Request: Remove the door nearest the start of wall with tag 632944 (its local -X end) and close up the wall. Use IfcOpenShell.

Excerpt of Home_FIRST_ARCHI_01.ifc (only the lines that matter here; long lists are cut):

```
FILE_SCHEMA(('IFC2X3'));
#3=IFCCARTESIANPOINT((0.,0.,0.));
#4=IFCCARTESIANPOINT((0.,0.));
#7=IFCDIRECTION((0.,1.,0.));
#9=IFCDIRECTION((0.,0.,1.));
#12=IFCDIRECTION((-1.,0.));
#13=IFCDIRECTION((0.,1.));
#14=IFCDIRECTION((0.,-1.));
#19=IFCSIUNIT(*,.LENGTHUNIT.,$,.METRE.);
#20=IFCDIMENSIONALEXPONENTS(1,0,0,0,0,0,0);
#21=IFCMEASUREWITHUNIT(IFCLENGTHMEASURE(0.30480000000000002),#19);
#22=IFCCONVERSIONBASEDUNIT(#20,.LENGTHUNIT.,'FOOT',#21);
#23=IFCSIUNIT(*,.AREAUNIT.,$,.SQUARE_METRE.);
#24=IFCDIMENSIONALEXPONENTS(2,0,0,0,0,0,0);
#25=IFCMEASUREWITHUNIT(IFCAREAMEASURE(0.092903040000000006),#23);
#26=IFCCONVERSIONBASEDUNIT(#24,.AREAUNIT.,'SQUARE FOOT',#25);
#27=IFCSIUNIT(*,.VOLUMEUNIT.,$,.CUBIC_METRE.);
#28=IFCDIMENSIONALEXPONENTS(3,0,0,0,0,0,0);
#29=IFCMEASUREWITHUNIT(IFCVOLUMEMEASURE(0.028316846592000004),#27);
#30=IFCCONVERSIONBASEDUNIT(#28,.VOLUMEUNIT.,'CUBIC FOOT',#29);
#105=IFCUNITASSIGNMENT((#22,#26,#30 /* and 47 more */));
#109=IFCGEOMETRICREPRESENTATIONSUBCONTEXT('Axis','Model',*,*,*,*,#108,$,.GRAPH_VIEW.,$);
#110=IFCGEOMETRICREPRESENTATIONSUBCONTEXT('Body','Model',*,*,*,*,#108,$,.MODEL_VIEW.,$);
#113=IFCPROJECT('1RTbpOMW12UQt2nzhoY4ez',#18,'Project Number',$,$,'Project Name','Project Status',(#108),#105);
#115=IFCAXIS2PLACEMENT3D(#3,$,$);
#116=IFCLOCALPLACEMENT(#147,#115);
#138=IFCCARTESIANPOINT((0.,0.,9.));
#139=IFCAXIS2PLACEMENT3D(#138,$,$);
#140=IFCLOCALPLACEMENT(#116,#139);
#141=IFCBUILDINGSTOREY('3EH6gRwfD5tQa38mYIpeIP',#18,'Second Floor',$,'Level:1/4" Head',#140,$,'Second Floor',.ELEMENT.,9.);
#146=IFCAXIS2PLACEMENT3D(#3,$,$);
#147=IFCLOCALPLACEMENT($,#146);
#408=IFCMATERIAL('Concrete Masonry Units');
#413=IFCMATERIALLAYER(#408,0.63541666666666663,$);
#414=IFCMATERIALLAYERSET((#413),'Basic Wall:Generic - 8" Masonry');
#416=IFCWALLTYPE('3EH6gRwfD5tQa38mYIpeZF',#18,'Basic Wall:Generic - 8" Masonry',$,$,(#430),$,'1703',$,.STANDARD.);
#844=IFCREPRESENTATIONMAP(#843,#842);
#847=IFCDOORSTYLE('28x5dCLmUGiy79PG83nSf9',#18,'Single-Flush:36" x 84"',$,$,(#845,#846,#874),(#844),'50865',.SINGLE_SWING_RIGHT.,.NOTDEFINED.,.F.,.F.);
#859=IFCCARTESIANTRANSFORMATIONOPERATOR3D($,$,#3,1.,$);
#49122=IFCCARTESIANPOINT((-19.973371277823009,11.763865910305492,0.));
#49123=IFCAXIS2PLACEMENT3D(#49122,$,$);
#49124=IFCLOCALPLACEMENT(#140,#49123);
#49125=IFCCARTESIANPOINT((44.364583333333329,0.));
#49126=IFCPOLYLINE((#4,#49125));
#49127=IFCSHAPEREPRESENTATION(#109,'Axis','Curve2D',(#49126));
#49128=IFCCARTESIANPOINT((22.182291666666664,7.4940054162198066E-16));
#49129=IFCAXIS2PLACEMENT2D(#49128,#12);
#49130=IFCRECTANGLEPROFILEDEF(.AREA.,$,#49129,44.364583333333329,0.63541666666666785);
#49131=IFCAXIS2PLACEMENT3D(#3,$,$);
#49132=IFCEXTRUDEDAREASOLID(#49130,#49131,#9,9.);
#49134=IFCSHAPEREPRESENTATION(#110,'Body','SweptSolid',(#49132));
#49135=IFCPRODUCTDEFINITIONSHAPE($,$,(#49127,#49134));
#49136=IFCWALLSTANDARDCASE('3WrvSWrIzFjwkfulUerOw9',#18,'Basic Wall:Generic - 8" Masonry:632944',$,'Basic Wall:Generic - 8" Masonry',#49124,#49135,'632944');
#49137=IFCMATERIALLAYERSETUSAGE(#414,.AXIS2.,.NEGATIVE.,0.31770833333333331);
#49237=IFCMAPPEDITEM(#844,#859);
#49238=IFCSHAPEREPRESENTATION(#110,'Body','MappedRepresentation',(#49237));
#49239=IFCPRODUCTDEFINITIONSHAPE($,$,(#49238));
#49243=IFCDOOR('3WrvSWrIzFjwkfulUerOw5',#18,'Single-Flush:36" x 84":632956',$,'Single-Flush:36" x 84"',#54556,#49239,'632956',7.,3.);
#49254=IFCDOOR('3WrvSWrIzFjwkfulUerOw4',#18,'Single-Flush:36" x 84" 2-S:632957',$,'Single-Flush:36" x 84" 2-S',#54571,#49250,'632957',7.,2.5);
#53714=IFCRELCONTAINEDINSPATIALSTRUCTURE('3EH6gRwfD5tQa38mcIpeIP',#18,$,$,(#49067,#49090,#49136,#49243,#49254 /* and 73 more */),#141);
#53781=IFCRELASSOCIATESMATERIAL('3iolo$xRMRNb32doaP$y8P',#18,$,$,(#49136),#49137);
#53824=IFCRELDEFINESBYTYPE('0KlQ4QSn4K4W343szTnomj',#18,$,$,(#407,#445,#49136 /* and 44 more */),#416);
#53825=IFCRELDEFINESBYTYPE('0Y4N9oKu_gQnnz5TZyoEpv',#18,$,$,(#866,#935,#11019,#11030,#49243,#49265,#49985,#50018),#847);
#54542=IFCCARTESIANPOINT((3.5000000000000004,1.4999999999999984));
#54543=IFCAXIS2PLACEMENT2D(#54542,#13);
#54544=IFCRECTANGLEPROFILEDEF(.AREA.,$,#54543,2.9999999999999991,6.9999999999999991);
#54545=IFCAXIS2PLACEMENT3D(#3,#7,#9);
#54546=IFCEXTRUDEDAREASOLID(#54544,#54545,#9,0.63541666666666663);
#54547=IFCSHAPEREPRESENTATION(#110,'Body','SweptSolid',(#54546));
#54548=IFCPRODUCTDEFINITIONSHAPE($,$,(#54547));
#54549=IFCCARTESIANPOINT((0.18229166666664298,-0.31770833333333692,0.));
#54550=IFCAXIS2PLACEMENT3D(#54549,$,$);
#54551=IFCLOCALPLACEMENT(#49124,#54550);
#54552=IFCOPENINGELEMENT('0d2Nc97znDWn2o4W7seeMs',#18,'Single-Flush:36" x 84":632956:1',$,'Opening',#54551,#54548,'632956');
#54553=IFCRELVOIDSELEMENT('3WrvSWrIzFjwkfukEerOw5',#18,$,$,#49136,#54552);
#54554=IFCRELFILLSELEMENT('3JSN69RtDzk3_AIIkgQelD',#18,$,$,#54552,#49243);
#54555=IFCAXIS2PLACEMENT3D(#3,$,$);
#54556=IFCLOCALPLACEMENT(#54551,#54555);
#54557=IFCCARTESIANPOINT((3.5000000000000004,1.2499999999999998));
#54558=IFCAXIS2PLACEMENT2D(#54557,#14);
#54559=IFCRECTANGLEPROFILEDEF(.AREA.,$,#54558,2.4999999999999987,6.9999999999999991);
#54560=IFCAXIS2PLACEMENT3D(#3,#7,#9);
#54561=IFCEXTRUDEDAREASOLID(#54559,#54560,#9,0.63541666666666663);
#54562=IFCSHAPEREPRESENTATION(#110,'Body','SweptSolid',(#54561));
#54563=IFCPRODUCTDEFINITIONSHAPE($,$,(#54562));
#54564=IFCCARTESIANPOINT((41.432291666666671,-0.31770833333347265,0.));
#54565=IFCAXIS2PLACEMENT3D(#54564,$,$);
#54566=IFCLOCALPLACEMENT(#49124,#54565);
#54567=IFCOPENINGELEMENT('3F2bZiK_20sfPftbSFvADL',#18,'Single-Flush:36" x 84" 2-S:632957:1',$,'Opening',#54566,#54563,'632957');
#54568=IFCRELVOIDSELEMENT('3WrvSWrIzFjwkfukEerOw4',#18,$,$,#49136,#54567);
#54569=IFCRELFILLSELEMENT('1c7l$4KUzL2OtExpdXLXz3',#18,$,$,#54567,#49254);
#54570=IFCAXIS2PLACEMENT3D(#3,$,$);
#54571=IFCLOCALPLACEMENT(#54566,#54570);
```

```python
import ifcopenshell
import ifcopenshell.api.feature
import ifcopenshell.api.root
import ifcopenshell.geom
import ifcopenshell.util.shape

model = ifcopenshell.open("Home_FIRST_ARCHI_01.ifc")
settings = ifcopenshell.geom.settings()


def volume(element):
    """Net volume in cubic metres, openings subtracted."""
    shape = ifcopenshell.geom.create_shape(settings, element)
    return ifcopenshell.util.shape.get_volume(shape.geometry)


door = model.by_id(49243)
opening = door.FillsVoids[0].RelatingOpeningElement
wall = opening.VoidsElements[0].RelatingBuildingElement
before = volume(wall)

ifcopenshell.api.root.remove_product(model, product=door)
ifcopenshell.api.feature.remove_feature(model, feature=opening)

after = volume(wall)

print(f"wall volume {before:.3f} -> {after:.3f} m3")

model.write("Home_FIRST_ARCHI_01-out.ifc")
```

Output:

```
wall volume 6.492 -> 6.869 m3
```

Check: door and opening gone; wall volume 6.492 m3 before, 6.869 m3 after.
